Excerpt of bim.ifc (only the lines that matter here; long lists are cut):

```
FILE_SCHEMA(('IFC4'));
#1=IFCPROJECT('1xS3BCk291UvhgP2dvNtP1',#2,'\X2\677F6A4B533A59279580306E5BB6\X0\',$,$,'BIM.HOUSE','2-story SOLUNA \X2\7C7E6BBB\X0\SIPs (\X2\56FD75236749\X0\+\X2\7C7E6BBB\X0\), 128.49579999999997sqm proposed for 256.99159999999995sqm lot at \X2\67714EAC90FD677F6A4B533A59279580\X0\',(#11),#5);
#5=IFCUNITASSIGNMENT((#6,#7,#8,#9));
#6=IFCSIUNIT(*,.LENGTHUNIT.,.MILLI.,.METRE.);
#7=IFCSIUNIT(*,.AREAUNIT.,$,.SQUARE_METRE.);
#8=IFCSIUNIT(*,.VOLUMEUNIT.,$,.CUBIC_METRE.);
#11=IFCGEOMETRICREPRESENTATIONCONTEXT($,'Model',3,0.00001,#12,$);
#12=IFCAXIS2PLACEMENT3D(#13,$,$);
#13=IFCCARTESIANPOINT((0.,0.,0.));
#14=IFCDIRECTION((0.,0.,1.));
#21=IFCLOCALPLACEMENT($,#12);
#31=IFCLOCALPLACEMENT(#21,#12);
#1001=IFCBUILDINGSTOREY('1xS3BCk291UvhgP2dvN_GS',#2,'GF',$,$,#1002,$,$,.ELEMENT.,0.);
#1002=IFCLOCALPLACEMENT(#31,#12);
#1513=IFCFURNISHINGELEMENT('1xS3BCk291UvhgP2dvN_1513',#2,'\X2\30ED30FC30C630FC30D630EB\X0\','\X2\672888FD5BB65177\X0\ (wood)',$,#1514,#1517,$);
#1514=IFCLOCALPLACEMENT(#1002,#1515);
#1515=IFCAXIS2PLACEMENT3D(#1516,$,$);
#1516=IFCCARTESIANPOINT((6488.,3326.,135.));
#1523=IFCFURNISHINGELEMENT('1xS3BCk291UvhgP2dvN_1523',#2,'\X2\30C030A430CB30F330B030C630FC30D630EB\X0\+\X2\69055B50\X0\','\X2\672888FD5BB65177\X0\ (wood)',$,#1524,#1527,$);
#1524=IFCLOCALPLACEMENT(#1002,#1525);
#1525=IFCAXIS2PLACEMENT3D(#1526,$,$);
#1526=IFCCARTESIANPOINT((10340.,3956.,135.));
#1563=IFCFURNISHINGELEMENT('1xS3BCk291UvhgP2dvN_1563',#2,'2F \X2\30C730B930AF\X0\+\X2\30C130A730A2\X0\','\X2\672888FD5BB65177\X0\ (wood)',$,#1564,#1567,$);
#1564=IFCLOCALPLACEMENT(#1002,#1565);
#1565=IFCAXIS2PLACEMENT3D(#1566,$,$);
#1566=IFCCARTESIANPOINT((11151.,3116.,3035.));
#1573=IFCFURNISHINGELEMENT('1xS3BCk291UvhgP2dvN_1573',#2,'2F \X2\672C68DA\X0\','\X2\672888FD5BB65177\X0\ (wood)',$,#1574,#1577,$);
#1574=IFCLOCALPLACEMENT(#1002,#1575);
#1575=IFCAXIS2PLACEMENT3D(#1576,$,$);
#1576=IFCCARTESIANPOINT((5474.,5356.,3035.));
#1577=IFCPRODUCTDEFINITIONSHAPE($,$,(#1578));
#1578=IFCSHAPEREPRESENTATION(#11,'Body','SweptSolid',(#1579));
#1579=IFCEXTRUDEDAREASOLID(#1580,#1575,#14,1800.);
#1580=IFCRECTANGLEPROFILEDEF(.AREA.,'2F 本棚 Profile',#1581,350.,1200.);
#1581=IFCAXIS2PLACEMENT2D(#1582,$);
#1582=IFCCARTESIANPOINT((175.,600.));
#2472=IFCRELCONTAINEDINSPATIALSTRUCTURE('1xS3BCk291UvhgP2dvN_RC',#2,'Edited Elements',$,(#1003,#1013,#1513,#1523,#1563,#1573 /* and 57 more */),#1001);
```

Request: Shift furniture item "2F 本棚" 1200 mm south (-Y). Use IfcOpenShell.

```python
import ifcopenshell
import ifcopenshell.api.geometry
import ifcopenshell.util.placement
import ifcopenshell.util.unit

model = ifcopenshell.open("bim.ifc")
unit_scale = ifcopenshell.util.unit.calculate_unit_scale(model)

item = model.by_guid("1xS3BCk291UvhgP2dvN_1573")
matrix = ifcopenshell.util.placement.get_local_placement(item.ObjectPlacement)
matrix[1, 3] -= 1.2 / unit_scale
ifcopenshell.api.geometry.edit_object_placement(model, product=item, matrix=matrix, is_si=False)

print(ifcopenshell.util.placement.get_local_placement(item.ObjectPlacement).round(3) + 0.0)

model.write("bim_rev.ifc")
```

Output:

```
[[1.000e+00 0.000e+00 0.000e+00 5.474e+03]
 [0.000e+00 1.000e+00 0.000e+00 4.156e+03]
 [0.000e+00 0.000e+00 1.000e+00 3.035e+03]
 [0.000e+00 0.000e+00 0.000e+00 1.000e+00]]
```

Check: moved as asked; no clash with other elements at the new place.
